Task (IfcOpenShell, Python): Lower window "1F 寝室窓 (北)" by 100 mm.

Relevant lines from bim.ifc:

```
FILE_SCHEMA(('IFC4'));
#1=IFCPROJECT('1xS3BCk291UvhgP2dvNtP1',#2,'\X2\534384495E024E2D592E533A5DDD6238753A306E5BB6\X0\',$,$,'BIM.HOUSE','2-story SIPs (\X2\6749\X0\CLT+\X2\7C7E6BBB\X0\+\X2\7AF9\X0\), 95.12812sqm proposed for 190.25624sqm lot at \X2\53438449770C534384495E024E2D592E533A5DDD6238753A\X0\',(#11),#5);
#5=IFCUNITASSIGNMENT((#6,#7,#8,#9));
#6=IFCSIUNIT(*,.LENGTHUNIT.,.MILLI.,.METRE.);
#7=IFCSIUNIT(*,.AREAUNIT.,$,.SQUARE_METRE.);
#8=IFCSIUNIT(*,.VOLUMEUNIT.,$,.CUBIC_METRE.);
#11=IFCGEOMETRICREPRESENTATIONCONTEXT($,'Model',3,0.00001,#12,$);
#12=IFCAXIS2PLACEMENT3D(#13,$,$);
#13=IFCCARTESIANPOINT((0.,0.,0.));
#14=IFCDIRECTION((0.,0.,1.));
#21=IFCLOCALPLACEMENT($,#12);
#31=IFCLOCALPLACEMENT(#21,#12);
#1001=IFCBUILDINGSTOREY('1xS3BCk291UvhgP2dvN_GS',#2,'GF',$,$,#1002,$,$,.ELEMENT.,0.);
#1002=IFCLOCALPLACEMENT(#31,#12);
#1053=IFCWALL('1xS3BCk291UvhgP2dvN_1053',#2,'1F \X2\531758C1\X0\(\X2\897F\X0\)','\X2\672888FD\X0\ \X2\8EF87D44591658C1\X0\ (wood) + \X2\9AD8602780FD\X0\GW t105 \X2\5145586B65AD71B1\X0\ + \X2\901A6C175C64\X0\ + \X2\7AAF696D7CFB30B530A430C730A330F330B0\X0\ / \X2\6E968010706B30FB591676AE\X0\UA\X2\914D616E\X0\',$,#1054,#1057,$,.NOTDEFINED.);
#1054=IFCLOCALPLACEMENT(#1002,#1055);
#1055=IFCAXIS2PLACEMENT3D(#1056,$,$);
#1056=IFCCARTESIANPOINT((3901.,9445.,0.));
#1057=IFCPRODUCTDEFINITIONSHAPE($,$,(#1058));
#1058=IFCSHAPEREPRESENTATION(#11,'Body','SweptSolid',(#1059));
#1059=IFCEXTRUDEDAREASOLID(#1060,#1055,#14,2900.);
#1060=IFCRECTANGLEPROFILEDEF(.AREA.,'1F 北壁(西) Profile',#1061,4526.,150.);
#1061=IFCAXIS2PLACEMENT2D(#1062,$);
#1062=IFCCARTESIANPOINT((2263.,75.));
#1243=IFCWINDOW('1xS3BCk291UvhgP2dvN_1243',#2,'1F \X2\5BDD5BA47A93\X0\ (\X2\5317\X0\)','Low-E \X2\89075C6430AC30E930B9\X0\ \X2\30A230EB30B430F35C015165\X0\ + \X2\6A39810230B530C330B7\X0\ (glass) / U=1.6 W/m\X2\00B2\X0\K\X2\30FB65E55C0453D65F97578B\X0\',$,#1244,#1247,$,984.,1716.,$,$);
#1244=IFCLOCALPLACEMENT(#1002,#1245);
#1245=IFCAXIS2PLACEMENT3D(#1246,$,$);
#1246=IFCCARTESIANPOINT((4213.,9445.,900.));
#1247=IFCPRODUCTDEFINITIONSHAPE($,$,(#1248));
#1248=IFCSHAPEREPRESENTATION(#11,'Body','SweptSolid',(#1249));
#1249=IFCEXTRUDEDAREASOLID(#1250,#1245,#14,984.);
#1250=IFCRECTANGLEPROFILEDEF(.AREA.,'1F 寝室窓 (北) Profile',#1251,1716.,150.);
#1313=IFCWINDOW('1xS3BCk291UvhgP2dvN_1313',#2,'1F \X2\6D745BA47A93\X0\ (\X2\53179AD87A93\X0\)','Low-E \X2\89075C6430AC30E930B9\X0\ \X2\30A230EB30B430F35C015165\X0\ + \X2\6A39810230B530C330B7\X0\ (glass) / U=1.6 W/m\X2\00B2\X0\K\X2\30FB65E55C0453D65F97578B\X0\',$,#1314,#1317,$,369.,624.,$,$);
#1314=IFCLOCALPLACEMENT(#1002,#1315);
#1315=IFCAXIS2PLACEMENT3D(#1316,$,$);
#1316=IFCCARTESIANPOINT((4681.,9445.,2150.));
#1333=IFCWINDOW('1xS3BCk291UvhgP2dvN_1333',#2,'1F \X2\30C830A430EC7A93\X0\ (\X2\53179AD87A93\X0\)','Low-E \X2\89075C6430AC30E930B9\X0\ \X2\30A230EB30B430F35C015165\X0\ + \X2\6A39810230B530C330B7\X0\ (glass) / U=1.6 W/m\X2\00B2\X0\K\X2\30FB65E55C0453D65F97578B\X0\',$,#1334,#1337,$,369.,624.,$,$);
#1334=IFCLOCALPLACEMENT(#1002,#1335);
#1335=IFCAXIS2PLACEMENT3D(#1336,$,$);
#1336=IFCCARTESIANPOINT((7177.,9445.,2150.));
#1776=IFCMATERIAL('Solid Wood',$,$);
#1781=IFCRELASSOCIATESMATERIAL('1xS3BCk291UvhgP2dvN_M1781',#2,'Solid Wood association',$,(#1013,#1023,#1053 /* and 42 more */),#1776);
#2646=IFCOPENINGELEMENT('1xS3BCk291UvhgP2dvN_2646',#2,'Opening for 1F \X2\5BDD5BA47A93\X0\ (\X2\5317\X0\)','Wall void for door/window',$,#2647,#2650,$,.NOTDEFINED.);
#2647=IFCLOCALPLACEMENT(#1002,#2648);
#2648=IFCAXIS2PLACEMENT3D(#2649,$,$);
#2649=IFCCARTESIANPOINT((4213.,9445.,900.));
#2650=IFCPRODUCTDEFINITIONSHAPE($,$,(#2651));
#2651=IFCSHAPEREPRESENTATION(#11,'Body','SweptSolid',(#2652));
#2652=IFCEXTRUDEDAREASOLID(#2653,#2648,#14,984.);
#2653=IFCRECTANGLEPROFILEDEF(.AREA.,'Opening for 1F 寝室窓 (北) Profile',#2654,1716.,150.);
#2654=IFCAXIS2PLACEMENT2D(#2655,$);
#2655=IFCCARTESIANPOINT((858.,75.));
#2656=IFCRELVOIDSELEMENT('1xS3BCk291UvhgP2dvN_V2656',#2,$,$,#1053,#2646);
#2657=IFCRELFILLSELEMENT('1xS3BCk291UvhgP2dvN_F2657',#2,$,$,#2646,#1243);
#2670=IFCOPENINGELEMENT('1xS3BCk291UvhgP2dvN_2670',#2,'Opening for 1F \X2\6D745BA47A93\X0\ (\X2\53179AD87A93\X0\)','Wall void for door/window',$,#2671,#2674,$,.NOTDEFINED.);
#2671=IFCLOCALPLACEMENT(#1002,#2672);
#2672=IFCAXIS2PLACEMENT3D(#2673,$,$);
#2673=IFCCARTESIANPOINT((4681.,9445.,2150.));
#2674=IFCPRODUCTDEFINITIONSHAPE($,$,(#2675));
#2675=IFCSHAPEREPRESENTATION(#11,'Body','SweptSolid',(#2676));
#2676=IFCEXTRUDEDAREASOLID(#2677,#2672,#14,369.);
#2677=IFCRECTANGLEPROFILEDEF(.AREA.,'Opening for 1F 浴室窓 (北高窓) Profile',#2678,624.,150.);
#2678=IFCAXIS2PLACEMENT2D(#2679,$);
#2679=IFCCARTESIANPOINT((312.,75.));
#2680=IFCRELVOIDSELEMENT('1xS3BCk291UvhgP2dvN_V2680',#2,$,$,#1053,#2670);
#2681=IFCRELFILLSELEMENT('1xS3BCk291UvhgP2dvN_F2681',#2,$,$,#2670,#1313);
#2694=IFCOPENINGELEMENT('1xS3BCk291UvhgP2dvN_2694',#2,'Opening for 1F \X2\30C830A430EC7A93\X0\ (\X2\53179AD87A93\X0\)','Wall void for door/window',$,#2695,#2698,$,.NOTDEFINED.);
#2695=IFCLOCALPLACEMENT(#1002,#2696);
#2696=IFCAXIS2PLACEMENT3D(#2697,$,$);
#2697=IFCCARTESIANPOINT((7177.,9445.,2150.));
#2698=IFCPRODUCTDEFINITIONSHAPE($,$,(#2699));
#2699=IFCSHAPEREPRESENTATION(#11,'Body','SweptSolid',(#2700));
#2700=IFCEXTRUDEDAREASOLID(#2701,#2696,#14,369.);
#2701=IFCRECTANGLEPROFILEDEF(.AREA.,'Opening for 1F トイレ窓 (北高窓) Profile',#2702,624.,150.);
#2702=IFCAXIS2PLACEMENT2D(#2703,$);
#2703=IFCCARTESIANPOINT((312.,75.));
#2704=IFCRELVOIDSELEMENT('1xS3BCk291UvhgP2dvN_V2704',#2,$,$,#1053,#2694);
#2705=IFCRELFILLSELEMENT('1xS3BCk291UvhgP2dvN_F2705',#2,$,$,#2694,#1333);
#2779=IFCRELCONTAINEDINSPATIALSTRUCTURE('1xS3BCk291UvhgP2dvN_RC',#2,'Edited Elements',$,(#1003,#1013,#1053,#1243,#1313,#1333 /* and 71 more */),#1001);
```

```python
import numpy as np
import ifcopenshell
import ifcopenshell.api.geometry
import ifcopenshell.util.placement
import ifcopenshell.util.unit

model = ifcopenshell.open("bim.ifc")
unit_scale = ifcopenshell.util.unit.calculate_unit_scale(model)

window = model.by_guid("1xS3BCk291UvhgP2dvN_1243")
opening = window.FillsVoids[0].RelatingOpeningElement
dz = -100.0

shift = np.array([0.0, 0.0, dz])
# The window is not placed relative to its opening, so move both.
for product in (opening, window):
    matrix = ifcopenshell.util.placement.get_local_placement(product.ObjectPlacement)
    matrix[:3, 3] += shift
    ifcopenshell.api.geometry.edit_object_placement(model, product=product, matrix=matrix, is_si=False)

print(f"moved by {dz * unit_scale:+.3f} m")

model.write("bim_v2.ifc")
```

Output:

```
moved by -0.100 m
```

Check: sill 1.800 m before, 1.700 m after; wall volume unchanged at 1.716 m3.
